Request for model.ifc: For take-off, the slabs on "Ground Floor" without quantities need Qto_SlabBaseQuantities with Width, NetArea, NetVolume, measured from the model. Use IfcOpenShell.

First a look at what the model holds.

```python
import ifcopenshell
import ifcopenshell.util.element
import ifcopenshell.util.unit

model = ifcopenshell.open("model.ifc")
print(model.schema)
for unit_type in ("LENGTHUNIT", "AREAUNIT", "VOLUMEUNIT"):
    print(unit_type, ifcopenshell.util.unit.calculate_unit_scale(model, unit_type))
storey = next(s for s in model.by_type("IfcBuildingStorey") if s.Name == "Ground Floor")
slabs = [e for e in ifcopenshell.util.element.get_decomposition(storey) if e.is_a("IfcSlab")]
for e in sorted(slabs, key=lambda e: e.id()):
    print(e.id(), e.is_a(), e.Name, list(ifcopenshell.util.element.get_psets(e, qtos_only=True)), sep=" | ")
```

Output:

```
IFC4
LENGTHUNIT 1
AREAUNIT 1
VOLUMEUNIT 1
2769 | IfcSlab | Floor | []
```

```python
import ifcopenshell
import ifcopenshell.api.pset
import ifcopenshell.geom
import ifcopenshell.util.element
import ifcopenshell.util.shape
import ifcopenshell.util.unit

model = ifcopenshell.open("model.ifc")
unit_scale = ifcopenshell.util.unit.calculate_unit_scale(model)
area_scale = ifcopenshell.util.unit.calculate_unit_scale(model, "AREAUNIT")
volume_scale = ifcopenshell.util.unit.calculate_unit_scale(model, "VOLUMEUNIT")
settings = ifcopenshell.geom.settings()

storey = next(s for s in model.by_type("IfcBuildingStorey") if s.Name == "Ground Floor")
slabs = [e for e in ifcopenshell.util.element.get_decomposition(storey) if e.is_a("IfcSlab")]

for e in sorted(slabs, key=lambda e: e.id()):
    if ifcopenshell.util.element.get_psets(e, qtos_only=True, should_inherit=False):
        continue
    # Geometry comes back in metres, in the element's own axes.
    shape = ifcopenshell.geom.create_shape(settings, e)
    values = {
        "Width": ifcopenshell.util.shape.get_z(shape.geometry) / unit_scale,
        "NetArea": ifcopenshell.util.shape.get_footprint_area(shape.geometry) / area_scale,
        "NetVolume": ifcopenshell.util.shape.get_volume(shape.geometry) / volume_scale,
    }
    qto = ifcopenshell.api.pset.add_qto(model, product=e, name="Qto_SlabBaseQuantities")
    ifcopenshell.api.pset.edit_qto(model, qto=qto, properties=values)
    print(e.id(), {k: round(v, 3) for k, v in values.items()})

model.write("model-out.ifc")
```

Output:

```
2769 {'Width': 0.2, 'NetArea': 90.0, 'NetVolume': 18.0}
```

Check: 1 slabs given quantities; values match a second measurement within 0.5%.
